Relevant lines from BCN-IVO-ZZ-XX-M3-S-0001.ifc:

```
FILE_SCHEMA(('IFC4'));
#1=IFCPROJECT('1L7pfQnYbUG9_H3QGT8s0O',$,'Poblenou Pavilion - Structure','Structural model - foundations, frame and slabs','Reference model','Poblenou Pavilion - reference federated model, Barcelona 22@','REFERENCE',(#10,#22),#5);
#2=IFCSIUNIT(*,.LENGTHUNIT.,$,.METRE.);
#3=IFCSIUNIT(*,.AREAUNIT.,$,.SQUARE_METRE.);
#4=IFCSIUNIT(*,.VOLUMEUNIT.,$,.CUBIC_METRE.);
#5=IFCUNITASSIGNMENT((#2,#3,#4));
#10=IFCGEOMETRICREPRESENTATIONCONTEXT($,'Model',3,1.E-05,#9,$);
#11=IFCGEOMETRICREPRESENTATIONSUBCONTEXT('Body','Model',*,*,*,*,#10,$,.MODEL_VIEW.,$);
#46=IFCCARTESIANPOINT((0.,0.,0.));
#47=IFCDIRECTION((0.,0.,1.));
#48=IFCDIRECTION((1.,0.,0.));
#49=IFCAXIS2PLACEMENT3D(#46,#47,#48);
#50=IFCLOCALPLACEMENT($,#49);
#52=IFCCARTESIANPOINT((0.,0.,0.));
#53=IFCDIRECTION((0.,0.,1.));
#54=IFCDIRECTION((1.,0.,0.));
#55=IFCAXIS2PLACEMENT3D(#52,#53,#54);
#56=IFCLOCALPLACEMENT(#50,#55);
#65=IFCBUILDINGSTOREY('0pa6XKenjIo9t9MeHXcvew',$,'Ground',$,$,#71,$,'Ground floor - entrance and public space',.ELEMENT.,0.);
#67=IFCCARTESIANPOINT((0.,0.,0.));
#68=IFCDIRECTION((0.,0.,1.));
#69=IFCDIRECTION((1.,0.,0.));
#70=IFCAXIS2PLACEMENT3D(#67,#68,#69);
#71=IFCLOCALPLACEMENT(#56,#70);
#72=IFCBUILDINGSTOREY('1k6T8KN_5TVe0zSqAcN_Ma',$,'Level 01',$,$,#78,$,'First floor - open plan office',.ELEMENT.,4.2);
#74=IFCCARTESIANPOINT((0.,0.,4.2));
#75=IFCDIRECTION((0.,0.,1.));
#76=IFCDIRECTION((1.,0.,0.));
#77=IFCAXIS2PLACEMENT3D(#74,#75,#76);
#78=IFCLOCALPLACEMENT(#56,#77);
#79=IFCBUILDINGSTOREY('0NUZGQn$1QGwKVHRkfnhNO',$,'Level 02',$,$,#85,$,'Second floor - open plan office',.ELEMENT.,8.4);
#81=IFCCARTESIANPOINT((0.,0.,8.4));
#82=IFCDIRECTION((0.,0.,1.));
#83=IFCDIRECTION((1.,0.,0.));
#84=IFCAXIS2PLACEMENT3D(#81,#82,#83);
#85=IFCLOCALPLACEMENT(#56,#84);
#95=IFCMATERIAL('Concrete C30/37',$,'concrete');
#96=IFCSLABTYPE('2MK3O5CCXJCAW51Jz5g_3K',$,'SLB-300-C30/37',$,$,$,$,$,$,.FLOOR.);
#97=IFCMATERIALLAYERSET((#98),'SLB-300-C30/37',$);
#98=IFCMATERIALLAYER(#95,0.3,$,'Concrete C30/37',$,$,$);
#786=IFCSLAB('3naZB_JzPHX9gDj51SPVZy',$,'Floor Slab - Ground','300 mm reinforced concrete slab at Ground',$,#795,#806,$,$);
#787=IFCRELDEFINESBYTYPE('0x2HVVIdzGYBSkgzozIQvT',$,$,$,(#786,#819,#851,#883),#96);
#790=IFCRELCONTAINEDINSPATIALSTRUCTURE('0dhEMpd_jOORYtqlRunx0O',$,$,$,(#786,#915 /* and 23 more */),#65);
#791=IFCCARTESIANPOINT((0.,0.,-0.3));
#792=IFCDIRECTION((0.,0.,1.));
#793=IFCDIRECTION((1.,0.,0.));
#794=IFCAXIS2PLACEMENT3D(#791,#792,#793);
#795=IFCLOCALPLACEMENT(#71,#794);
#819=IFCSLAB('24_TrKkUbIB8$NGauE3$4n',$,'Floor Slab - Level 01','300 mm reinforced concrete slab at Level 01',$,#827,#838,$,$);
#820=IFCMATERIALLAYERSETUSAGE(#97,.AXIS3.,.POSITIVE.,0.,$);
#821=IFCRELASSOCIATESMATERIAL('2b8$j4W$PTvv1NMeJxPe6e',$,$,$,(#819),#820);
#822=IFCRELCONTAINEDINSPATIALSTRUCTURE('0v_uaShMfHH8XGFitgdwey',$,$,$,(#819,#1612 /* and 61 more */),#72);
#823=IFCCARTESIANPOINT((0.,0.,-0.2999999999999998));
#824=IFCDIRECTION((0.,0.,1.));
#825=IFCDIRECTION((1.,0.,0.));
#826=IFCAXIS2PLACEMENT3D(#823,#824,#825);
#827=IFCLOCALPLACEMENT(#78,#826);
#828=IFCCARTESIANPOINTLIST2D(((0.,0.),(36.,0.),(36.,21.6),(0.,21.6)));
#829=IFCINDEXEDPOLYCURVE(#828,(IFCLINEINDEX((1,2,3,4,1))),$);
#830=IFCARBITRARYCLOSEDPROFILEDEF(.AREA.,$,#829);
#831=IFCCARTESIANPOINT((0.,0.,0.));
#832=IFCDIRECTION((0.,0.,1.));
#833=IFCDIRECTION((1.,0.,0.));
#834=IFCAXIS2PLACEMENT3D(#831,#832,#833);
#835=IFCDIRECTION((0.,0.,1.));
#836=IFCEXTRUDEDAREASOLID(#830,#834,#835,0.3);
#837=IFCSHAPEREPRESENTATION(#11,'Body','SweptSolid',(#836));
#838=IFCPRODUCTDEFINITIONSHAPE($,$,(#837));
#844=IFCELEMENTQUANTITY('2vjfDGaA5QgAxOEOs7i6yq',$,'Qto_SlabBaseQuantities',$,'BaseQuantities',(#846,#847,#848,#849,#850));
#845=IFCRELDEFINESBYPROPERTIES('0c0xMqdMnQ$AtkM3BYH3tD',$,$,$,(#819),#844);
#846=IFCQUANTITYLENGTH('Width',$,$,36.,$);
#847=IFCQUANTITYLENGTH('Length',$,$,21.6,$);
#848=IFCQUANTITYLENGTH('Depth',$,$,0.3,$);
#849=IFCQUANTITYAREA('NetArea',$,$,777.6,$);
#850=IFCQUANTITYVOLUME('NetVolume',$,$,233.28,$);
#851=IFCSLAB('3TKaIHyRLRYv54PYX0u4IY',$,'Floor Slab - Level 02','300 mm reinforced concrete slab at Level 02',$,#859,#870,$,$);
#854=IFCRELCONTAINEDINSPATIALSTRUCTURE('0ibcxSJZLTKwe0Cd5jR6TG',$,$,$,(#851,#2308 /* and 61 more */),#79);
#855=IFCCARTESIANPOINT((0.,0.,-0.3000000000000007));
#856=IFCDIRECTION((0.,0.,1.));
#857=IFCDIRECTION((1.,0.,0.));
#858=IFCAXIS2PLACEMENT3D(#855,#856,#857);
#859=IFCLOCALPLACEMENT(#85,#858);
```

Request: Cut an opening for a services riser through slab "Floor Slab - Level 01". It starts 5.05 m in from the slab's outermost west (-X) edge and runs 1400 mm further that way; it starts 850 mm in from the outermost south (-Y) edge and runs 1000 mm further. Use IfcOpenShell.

```python
import numpy as np
import ifcopenshell
import ifcopenshell.api.feature
import ifcopenshell.api.geometry
import ifcopenshell.api.pset
import ifcopenshell.api.root
import ifcopenshell.geom
import ifcopenshell.util.element
import ifcopenshell.util.placement
import ifcopenshell.util.representation
import ifcopenshell.util.shape
import ifcopenshell.util.unit

model = ifcopenshell.open("BCN-IVO-ZZ-XX-M3-S-0001.ifc")
unit_scale = ifcopenshell.util.unit.calculate_unit_scale(model)
area_scale = ifcopenshell.util.unit.calculate_unit_scale(model, "AREAUNIT")
volume_scale = ifcopenshell.util.unit.calculate_unit_scale(model, "VOLUMEUNIT")
settings = ifcopenshell.geom.settings()


def volume(element):
    """Net volume in cubic metres, openings subtracted."""
    shape = ifcopenshell.geom.create_shape(settings, element)
    return ifcopenshell.util.shape.get_volume(shape.geometry)


slab = model.by_guid("24_TrKkUbIB8$NGauE3$4n")
before = volume(slab)

# Extent in the slab's own axes, in metres. The edges named are its -X and -Y sides.
slab_shape = ifcopenshell.geom.create_shape(settings, slab)
vertices = ifcopenshell.util.shape.get_vertices(slab_shape.geometry)
x_min, y_min, bottom = vertices.min(axis=0)
top = vertices[:, 2].max()

opening = ifcopenshell.api.root.create_entity(model, ifc_class="IfcOpeningElement", name="Services riser opening", predefined_type="OPENING")
context = ifcopenshell.util.representation.get_context(model, "Model", "Body", "MODEL_VIEW")
width, depth = 1.4, 1
outline = [(0.0, 0.0), (width, 0.0), (width, depth), (0.0, depth), (0.0, 0.0)]
# Overshoot both faces by 50 mm so the cut is clean.
shape = ifcopenshell.api.geometry.add_slab_representation(
    model, context=context, depth=top - bottom + 0.1, polyline=outline
)
ifcopenshell.api.geometry.assign_representation(model, product=opening, representation=shape)

matrix = ifcopenshell.util.placement.get_local_placement(slab.ObjectPlacement)
matrix[:, 3] = matrix @ np.append(np.array([x_min + 5.05, y_min + 0.85, bottom - 0.05]) / unit_scale, 1.0)
ifcopenshell.api.geometry.edit_object_placement(model, product=opening, matrix=matrix, is_si=False)
ifcopenshell.api.feature.add_feature(model, feature=opening, element=slab)

after = volume(slab)

# Update the slab's stored quantities.
qto = model.by_id(ifcopenshell.util.element.get_pset(slab, "Qto_SlabBaseQuantities", should_inherit=False)["id"])
ifcopenshell.api.pset.edit_qto(model, qto=qto, properties={
    "NetArea": after / (top - bottom) / area_scale,
    "NetVolume": after / volume_scale,
})

print(f"slab volume {before:.3f} -> {after:.3f} m3")

model.write("BCN-IVO-ZZ-XX-M3-S-0001-out.ifc")
```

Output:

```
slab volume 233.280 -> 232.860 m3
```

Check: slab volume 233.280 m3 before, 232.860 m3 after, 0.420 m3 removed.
